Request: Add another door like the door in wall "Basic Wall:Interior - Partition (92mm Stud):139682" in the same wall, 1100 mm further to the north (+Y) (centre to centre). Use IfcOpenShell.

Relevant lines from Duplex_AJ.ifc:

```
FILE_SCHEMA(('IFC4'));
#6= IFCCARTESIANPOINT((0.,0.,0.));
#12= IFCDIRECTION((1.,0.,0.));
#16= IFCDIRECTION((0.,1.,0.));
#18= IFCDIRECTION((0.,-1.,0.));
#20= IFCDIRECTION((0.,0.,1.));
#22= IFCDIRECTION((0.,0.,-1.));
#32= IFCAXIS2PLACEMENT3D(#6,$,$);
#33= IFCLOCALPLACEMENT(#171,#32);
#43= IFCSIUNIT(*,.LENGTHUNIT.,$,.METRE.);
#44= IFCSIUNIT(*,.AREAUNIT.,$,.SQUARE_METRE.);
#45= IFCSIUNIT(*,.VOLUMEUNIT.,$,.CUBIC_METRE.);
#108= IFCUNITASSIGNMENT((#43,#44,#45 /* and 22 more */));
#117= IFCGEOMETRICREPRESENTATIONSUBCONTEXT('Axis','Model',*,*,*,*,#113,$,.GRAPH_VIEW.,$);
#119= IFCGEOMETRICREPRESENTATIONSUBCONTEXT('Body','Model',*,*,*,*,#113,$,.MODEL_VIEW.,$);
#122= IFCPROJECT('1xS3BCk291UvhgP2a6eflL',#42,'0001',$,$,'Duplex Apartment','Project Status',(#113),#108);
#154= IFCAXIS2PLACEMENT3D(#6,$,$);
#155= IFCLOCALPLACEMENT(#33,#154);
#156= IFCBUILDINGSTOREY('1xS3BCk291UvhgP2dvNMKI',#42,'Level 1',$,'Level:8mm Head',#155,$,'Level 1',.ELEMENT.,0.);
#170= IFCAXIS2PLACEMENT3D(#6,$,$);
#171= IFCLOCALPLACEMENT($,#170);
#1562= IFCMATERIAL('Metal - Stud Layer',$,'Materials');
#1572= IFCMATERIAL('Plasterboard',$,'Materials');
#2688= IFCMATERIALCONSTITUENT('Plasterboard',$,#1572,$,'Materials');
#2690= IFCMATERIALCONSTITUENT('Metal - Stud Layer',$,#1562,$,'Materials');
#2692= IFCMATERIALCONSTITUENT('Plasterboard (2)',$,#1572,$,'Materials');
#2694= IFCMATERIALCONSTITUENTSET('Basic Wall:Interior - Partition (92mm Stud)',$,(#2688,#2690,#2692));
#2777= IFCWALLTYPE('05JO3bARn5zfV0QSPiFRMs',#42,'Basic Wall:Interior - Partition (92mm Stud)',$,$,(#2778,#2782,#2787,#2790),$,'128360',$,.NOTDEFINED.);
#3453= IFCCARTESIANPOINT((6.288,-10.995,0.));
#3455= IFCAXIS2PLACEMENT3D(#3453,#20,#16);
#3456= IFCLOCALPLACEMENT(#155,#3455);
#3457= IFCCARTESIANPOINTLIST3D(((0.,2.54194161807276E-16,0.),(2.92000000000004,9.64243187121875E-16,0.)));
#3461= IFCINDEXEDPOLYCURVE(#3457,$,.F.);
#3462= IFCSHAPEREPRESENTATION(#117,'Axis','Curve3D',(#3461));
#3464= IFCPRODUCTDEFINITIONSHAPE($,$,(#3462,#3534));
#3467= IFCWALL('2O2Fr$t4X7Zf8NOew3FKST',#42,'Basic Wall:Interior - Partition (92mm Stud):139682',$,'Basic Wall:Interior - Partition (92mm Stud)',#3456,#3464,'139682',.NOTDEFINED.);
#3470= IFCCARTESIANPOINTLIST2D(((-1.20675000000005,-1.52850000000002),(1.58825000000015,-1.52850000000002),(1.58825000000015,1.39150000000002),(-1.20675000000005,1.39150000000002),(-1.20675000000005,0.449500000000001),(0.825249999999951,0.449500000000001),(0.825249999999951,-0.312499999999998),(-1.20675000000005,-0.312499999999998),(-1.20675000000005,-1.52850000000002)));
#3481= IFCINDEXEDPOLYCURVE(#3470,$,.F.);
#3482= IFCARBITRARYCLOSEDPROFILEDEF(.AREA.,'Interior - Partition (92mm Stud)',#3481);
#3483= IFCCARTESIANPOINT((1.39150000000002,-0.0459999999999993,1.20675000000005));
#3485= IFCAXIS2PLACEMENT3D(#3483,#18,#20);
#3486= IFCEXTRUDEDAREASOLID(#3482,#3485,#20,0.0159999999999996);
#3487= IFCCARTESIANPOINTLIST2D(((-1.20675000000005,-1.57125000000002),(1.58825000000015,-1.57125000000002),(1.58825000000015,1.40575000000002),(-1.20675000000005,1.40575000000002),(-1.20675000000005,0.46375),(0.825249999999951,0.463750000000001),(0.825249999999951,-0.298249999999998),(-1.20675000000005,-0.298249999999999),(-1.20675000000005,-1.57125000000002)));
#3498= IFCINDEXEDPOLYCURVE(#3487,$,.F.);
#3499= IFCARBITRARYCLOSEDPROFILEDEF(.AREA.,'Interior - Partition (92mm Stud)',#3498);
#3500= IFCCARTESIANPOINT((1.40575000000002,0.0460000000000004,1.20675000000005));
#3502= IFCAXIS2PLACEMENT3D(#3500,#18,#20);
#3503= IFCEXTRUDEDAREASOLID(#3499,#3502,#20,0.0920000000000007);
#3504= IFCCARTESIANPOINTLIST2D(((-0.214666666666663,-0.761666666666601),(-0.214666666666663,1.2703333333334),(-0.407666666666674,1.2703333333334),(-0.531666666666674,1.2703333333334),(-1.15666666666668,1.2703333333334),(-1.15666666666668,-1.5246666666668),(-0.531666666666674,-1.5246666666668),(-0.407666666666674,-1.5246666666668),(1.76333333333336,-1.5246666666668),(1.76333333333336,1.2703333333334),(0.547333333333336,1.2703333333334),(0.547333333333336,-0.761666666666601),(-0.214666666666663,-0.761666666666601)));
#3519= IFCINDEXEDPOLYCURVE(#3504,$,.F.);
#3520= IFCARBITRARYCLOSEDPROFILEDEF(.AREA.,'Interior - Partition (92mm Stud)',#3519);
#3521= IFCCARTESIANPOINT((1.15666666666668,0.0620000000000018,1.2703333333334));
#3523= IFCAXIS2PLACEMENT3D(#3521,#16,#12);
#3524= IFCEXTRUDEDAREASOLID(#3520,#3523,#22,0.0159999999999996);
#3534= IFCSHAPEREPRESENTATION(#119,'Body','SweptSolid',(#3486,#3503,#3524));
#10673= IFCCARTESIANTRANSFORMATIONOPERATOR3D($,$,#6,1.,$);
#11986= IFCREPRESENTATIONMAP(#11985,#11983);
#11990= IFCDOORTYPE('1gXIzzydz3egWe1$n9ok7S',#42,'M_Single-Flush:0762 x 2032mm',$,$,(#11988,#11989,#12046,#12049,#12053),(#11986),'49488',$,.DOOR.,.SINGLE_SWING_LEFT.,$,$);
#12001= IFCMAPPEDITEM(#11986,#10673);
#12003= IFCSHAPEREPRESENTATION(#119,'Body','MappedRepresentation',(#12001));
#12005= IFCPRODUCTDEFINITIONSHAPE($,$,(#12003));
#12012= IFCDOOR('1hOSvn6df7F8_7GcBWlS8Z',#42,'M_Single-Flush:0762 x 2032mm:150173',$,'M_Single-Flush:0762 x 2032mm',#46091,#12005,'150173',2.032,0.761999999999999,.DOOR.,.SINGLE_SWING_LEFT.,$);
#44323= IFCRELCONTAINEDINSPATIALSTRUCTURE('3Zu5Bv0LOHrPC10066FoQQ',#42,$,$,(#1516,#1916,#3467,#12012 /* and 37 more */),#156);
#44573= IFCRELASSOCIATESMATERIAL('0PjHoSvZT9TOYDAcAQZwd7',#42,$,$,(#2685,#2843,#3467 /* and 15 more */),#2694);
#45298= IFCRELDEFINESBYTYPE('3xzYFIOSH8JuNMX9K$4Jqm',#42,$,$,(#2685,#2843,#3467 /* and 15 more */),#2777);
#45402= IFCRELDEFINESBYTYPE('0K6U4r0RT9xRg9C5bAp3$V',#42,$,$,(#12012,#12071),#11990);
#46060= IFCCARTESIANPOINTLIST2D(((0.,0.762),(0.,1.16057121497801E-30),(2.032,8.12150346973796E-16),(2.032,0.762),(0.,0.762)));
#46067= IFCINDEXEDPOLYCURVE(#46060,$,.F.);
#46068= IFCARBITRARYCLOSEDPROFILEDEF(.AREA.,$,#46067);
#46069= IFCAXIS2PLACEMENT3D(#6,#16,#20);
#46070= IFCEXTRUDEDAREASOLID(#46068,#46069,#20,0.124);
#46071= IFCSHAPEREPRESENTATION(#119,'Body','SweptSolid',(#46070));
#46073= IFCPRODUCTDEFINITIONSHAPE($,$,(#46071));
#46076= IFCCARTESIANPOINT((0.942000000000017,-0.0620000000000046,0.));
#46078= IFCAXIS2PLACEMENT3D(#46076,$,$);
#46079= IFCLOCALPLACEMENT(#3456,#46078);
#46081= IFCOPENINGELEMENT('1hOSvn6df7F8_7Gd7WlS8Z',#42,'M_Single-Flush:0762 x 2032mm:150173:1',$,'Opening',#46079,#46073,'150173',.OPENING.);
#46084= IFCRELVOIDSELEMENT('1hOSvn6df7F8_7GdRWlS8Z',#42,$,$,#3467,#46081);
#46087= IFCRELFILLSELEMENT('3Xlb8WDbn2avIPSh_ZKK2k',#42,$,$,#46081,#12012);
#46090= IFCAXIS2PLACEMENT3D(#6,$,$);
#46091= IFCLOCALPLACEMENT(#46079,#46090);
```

```python
import ifcopenshell
import ifcopenshell.api.feature
import ifcopenshell.api.geometry
import ifcopenshell.api.root
import ifcopenshell.geom
import ifcopenshell.util.element
import ifcopenshell.util.placement
import ifcopenshell.util.shape

model = ifcopenshell.open("Duplex_AJ.ifc")
settings = ifcopenshell.geom.settings()


def volume(element):
    """Net volume in cubic metres, openings subtracted."""
    shape = ifcopenshell.geom.create_shape(settings, element)
    return ifcopenshell.util.shape.get_volume(shape.geometry)


def reuse_history(source, copy):
    """copy_class also copies each property set's owner history, people and application; keep the originals."""
    for rel in copy.IsDefinedBy:
        if rel.is_a("IfcRelDefinesByProperties") and (history := rel.RelatingPropertyDefinition.OwnerHistory):
            rel.RelatingPropertyDefinition.OwnerHistory = source.OwnerHistory
            ifcopenshell.util.element.remove_deep2(model, history)


door = model.by_guid("1hOSvn6df7F8_7GcBWlS8Z")
opening = door.FillsVoids[0].RelatingOpeningElement
wall = opening.VoidsElements[0].RelatingBuildingElement
before = volume(wall)
shift = ifcopenshell.util.placement.get_local_placement(wall.ObjectPlacement)[:3, 0] * 1.1

# copy_class copies the void relationship, type, container and properties, but no geometry.
new_opening = ifcopenshell.api.root.copy_class(model, product=opening)
new_opening.Representation = ifcopenshell.util.element.copy_deep(
    model, opening.Representation, exclude=["IfcGeometricRepresentationContext", "IfcRepresentationMap"]
)
new_opening.Name = "M_Single-Flush:0762 x 2032mm"
new_opening.Tag = None
new_door = ifcopenshell.api.root.copy_class(model, product=door)
new_door.Representation = ifcopenshell.util.element.copy_deep(
    model, door.Representation, exclude=["IfcGeometricRepresentationContext", "IfcRepresentationMap"]
)
new_door.Name = "M_Single-Flush:0762 x 2032mm"
new_door.Tag = None
reuse_history(door, new_door)
ifcopenshell.api.feature.add_filling(model, opening=new_opening, element=new_door)

for old, new in ((opening, new_opening), (door, new_door)):
    matrix = ifcopenshell.util.placement.get_local_placement(old.ObjectPlacement)
    matrix[:3, 3] += shift
    ifcopenshell.api.geometry.edit_object_placement(model, product=new, matrix=matrix, is_si=False)

after = volume(wall)

print(f"wall volume {before:.3f} -> {after:.3f} m3")

model.write("Duplex_AJ_rev.ifc")
```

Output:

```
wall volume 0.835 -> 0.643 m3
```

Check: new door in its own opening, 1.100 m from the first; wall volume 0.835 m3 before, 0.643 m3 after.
